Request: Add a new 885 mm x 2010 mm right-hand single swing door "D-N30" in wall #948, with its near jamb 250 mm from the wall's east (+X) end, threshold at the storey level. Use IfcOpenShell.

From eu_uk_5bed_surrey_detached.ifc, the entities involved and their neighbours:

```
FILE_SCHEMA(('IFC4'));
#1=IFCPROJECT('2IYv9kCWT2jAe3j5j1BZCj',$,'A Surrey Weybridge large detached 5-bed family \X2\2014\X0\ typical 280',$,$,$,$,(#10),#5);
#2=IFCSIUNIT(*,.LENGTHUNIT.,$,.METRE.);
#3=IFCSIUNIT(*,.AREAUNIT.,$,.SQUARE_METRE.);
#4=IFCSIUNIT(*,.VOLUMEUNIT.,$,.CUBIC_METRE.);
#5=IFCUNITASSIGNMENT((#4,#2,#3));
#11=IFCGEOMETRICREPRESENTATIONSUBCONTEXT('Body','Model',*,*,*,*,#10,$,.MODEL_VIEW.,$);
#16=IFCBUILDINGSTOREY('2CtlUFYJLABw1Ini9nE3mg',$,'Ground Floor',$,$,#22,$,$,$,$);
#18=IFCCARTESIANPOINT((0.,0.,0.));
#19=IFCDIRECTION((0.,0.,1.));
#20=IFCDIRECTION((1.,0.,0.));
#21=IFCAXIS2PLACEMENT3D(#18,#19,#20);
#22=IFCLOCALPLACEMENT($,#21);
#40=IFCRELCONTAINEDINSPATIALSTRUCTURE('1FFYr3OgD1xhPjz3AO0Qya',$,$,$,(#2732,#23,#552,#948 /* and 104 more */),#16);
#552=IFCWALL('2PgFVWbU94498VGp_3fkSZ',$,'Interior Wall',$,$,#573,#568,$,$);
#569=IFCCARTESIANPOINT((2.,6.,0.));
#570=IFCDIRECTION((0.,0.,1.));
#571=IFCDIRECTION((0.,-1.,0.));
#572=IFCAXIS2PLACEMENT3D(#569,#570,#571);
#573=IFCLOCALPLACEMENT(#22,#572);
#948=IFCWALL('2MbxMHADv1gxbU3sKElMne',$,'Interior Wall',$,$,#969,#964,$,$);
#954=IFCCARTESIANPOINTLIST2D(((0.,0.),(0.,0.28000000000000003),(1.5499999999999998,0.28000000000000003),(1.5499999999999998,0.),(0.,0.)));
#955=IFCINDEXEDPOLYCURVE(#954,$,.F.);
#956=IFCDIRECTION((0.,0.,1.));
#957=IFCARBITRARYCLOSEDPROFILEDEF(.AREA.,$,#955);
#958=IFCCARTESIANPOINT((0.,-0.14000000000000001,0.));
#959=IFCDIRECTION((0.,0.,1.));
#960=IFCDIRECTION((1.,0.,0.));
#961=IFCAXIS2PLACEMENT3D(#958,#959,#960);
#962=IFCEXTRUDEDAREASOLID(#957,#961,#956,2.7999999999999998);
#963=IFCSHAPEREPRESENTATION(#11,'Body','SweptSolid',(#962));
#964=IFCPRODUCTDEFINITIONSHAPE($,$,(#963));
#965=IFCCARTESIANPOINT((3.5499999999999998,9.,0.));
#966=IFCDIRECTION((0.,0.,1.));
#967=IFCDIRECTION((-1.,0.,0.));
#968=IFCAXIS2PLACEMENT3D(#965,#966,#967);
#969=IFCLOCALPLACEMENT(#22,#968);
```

```python
import numpy as np
import ifcopenshell
import ifcopenshell.api.feature
import ifcopenshell.api.geometry
import ifcopenshell.api.root
import ifcopenshell.api.spatial
import ifcopenshell.geom
import ifcopenshell.util.element
import ifcopenshell.util.placement
import ifcopenshell.util.representation
import ifcopenshell.util.shape
import ifcopenshell.util.unit

model = ifcopenshell.open("eu_uk_5bed_surrey_detached.ifc")
unit_scale = ifcopenshell.util.unit.calculate_unit_scale(model)
settings = ifcopenshell.geom.settings()


def volume(element):
    """Net volume in cubic metres, openings subtracted."""
    shape = ifcopenshell.geom.create_shape(settings, element)
    return ifcopenshell.util.shape.get_volume(shape.geometry)


wall = model.by_id(948)
storey = ifcopenshell.util.element.get_container(wall, ifc_class="IfcBuildingStorey")
context = ifcopenshell.util.representation.get_context(model, "Model", "Body", "MODEL_VIEW")
before = volume(wall)

width, height, from_end, sill = 0.885, 2.01, 0.25, 0.0  # metres

# The wall runs along its own X axis, and the end named is its -X end.
wall_shape = ifcopenshell.geom.create_shape(settings, wall)
x, y, z = ifcopenshell.util.shape.get_vertices(wall_shape.geometry).T
start = x.min() + from_end
face, thickness = float(y.min()), float(y.max() - y.min())
wall_matrix = ifcopenshell.util.placement.get_local_placement(wall.ObjectPlacement)
level = ifcopenshell.util.placement.get_local_placement(storey.ObjectPlacement)[2, 3]


def in_wall(x, y):
    """Placement at x, y metres in the wall's axes, at sill height."""
    matrix = wall_matrix.copy()
    matrix[:, 3] = wall_matrix @ np.array([x / unit_scale, y / unit_scale, 0.0, 1.0])
    matrix[2, 3] = level + sill / unit_scale
    return matrix


# Opening: a box that overshoots both wall faces by 50 mm.
opening = ifcopenshell.api.root.create_entity(model, ifc_class="IfcOpeningElement", predefined_type="OPENING")
box = ifcopenshell.api.geometry.add_wall_representation(
    model, context=context, length=width, height=height, thickness=thickness + 0.1
)
ifcopenshell.api.geometry.assign_representation(model, product=opening, representation=box)
ifcopenshell.api.geometry.edit_object_placement(model, product=opening, matrix=in_wall(start, face - 0.05), is_si=False)
ifcopenshell.api.feature.add_feature(model, feature=opening, element=wall)

door = ifcopenshell.api.root.create_entity(model, ifc_class="IfcDoor", name="D-N30", predefined_type="DOOR")
door.OverallWidth, door.OverallHeight = width / unit_scale, height / unit_scale
door.OperationType = "SINGLE_SWING_RIGHT"
body = ifcopenshell.api.geometry.add_door_representation(
    model,
    context=context,
    overall_width=door.OverallWidth,
    overall_height=door.OverallHeight,
    operation_type="SINGLE_SWING_RIGHT",
    lining_properties={"LiningDepth": thickness / unit_scale, "ThresholdDepth": thickness / unit_scale},
)
ifcopenshell.api.geometry.assign_representation(model, product=door, representation=body)
ifcopenshell.api.spatial.assign_container(model, products=[door], relating_structure=storey)
ifcopenshell.api.feature.add_filling(model, opening=opening, element=door)

# The lining spans the wall, so the door starts at the wall face.
ifcopenshell.api.geometry.edit_object_placement(model, product=door, matrix=in_wall(start, face), is_si=False)

after = volume(wall)

print(f"wall volume {before:.3f} -> {after:.3f} m3")

model.write("eu_uk_5bed_surrey_detached-out.ifc")
```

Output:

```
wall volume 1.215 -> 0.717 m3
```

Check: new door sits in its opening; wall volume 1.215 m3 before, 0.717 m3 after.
